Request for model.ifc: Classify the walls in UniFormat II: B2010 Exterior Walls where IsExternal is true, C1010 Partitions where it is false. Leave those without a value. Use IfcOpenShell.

First a look at what the model holds.

```python
import ifcopenshell
import ifcopenshell.util.element

model = ifcopenshell.open("model.ifc")
print(model.schema)
print("classifications:", [c.Name for c in model.by_type("IfcClassification")])
values = [ifcopenshell.util.element.get_pset(e, "Pset_WallCommon", "IsExternal") for e in model.by_type("IfcWall")]
for value in (True, False, None):
    print("IsExternal", value, values.count(value))
```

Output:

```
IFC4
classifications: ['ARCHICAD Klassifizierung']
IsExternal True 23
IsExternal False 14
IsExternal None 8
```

```python
import ifcopenshell
import ifcopenshell.api.classification
import ifcopenshell.util.element

model = ifcopenshell.open("model.ifc")

system = ifcopenshell.api.classification.add_classification(model, classification="UniFormat II")

walls = model.by_type("IfcWall")
external = {e: ifcopenshell.util.element.get_pset(e, "Pset_WallCommon", "IsExternal") for e in walls}
for flag, code, name in ((True, "B2010", "Exterior Walls"), (False, "C1010", "Partitions")):
    products = [e for e in walls if external[e] is flag]
    ifcopenshell.api.classification.add_reference(
        model, products=products, classification=system, identification=code, name=name
    )
    print(code, len(products))

model.write("model_edited.ifc")
```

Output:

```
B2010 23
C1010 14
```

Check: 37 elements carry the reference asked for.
